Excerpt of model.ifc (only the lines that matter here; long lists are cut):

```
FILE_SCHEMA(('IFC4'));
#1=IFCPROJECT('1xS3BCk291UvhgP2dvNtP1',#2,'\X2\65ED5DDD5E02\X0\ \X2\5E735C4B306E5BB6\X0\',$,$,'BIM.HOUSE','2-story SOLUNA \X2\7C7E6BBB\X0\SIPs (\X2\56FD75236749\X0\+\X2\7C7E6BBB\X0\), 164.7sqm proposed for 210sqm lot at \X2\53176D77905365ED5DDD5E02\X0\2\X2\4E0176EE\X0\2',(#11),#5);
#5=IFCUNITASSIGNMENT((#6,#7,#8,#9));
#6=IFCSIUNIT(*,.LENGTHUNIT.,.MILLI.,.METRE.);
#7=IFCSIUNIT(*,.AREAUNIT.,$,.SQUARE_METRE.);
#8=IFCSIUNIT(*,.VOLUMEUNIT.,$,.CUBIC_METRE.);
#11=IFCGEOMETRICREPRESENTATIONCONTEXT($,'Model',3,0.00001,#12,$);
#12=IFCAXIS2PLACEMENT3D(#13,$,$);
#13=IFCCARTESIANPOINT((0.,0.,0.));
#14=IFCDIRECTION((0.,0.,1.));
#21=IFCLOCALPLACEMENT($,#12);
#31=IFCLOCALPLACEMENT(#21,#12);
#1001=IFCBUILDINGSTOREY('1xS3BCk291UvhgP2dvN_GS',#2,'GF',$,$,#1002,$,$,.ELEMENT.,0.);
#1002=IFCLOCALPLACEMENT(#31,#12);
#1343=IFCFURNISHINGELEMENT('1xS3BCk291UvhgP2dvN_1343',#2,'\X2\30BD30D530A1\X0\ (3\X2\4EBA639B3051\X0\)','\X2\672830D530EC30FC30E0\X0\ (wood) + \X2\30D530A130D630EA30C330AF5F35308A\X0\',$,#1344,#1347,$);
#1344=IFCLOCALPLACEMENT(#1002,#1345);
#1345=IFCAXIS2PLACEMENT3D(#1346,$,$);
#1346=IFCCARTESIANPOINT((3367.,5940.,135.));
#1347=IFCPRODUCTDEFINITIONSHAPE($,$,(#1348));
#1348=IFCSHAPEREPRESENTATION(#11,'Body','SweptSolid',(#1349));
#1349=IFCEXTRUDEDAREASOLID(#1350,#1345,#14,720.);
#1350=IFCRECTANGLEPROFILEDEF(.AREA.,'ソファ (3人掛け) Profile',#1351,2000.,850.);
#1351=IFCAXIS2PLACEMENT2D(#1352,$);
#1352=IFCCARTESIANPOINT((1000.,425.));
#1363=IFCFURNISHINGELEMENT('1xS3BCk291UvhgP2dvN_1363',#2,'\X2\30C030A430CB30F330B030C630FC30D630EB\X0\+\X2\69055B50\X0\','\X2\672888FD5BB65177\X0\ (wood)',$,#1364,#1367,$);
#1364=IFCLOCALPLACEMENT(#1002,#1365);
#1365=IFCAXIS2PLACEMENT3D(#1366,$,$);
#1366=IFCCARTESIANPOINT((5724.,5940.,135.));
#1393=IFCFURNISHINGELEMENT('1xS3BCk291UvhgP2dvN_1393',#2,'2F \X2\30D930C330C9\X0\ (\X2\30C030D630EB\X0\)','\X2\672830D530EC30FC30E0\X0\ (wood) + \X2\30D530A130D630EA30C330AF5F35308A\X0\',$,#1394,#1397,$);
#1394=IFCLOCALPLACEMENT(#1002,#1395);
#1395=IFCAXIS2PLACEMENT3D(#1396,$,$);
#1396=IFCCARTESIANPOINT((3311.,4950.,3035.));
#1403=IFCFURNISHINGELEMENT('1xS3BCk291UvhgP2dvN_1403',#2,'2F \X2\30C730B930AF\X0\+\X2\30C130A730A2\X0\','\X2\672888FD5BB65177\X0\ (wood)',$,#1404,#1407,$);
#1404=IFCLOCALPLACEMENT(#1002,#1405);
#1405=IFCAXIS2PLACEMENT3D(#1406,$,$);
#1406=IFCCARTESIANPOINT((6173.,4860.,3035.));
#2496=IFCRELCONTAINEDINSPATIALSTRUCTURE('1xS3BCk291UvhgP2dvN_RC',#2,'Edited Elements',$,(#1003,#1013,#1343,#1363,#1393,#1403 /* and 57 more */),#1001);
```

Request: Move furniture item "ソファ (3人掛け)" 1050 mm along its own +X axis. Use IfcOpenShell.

```python
import ifcopenshell
import ifcopenshell.api.geometry
import ifcopenshell.util.placement

model = ifcopenshell.open("model.ifc")

item = model.by_guid("1xS3BCk291UvhgP2dvN_1343")
matrix = ifcopenshell.util.placement.get_local_placement(item.ObjectPlacement)
matrix[:3, 3] += matrix[:3, 0] * 1050.0
ifcopenshell.api.geometry.edit_object_placement(model, product=item, matrix=matrix, is_si=False)

print(ifcopenshell.util.placement.get_local_placement(item.ObjectPlacement).round(3) + 0.0)

model.write("model_rev.ifc")
```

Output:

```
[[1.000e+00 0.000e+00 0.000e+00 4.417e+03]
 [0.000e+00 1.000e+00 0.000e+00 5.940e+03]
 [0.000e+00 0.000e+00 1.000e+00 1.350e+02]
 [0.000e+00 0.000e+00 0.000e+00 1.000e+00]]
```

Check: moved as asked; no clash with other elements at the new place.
